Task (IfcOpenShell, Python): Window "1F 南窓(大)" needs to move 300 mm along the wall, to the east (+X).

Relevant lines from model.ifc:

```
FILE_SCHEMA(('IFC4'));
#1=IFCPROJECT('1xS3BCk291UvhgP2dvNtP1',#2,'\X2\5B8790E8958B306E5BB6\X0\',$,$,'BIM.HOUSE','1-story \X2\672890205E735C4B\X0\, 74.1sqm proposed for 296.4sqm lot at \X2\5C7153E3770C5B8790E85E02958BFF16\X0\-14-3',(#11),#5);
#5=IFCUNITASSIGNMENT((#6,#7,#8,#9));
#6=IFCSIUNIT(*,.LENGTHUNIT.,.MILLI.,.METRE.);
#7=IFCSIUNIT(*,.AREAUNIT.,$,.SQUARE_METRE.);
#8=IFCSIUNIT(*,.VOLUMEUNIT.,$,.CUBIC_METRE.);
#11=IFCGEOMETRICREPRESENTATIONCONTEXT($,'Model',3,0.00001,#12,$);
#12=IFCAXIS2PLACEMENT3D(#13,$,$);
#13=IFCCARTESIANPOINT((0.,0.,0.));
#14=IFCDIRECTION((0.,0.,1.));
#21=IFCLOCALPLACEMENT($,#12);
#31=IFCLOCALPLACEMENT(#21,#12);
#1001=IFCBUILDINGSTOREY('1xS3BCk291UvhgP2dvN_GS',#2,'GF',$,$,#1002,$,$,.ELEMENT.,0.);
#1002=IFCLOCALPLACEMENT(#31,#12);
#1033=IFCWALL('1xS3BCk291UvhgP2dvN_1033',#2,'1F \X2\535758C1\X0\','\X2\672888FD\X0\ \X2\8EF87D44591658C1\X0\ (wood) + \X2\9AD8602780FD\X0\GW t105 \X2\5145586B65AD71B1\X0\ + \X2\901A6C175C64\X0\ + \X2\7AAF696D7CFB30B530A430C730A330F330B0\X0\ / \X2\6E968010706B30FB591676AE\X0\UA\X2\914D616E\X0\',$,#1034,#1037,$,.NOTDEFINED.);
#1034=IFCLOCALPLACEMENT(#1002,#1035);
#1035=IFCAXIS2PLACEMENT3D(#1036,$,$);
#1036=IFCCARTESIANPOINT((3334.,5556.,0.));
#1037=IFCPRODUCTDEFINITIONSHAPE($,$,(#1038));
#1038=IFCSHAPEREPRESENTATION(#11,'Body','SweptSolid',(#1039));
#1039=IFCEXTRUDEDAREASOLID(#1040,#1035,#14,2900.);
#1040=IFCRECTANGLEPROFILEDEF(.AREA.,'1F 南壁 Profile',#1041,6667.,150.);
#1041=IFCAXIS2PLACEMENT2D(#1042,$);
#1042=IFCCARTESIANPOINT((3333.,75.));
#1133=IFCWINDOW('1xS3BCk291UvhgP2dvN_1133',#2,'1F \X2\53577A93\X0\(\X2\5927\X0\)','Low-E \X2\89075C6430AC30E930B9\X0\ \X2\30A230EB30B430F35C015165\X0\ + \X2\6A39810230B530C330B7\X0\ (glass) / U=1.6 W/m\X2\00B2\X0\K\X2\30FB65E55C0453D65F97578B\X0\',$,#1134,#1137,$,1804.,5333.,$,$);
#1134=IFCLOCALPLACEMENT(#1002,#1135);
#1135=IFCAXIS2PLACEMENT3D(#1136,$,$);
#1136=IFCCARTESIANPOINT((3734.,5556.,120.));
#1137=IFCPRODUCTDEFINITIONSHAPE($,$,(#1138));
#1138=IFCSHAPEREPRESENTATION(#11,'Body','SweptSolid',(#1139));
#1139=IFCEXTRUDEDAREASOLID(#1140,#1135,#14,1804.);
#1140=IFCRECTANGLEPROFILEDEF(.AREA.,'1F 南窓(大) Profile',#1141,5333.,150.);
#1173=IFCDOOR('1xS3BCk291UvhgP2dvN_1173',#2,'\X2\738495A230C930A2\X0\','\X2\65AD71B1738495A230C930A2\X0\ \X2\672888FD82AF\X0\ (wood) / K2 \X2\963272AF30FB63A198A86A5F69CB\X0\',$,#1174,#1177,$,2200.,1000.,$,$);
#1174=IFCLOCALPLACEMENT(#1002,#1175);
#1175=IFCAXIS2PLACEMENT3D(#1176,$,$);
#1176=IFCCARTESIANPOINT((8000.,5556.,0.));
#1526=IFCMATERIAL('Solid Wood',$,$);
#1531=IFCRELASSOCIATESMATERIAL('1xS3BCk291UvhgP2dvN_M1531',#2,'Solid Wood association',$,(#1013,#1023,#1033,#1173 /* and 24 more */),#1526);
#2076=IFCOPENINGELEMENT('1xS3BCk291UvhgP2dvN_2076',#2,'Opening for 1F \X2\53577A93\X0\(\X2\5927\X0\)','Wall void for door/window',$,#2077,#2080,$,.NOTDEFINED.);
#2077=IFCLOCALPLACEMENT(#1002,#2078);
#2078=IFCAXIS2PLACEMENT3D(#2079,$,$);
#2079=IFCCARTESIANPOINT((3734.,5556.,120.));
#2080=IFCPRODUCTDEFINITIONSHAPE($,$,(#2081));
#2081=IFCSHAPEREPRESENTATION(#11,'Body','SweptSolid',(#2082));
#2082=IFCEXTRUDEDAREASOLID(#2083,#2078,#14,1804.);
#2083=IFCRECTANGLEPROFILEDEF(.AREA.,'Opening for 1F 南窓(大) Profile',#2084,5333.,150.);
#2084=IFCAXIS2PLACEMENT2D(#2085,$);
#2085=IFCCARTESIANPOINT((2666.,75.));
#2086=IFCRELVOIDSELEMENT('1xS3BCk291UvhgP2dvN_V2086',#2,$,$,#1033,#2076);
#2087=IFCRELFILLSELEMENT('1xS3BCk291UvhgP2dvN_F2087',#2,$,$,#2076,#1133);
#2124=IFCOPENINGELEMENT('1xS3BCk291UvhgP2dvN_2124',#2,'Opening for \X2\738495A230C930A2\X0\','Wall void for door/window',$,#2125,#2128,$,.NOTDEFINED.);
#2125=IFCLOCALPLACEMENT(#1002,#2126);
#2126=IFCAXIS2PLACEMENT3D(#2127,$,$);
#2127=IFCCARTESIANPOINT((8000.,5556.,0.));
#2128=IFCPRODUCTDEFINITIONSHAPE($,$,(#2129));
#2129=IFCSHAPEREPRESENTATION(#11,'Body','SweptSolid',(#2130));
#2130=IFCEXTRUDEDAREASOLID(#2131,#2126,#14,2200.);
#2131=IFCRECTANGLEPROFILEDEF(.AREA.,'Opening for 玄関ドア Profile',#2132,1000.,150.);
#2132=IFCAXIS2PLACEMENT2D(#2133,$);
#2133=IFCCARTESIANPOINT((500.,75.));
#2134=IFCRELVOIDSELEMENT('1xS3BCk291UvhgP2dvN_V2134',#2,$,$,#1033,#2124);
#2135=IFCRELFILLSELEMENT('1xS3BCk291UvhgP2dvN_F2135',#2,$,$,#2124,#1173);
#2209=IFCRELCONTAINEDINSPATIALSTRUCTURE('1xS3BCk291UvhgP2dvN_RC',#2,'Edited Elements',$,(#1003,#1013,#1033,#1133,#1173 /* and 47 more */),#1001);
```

```python
import ifcopenshell
import ifcopenshell.api.geometry
import ifcopenshell.util.placement

model = ifcopenshell.open("model.ifc")

window = model.by_id(1133)
opening = window.FillsVoids[0].RelatingOpeningElement
wall = opening.VoidsElements[0].RelatingBuildingElement

wall_matrix = ifcopenshell.util.placement.get_local_placement(wall.ObjectPlacement)
shift = wall_matrix[:3, 0] * 300.0
before = ifcopenshell.util.placement.get_local_placement(window.ObjectPlacement)[:3, 3].copy()

# The window is not placed relative to its opening, so move both.
for product in (opening, window):
    matrix = ifcopenshell.util.placement.get_local_placement(product.ObjectPlacement)
    matrix[:3, 3] += shift
    ifcopenshell.api.geometry.edit_object_placement(model, product=product, matrix=matrix, is_si=False)

after = ifcopenshell.util.placement.get_local_placement(window.ObjectPlacement)[:3, 3]
print("window moved by", (after - before).round(3) + 0.0)

model.write("model_updated.ifc")
```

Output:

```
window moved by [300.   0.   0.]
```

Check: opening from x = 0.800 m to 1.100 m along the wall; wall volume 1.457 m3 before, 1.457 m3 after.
